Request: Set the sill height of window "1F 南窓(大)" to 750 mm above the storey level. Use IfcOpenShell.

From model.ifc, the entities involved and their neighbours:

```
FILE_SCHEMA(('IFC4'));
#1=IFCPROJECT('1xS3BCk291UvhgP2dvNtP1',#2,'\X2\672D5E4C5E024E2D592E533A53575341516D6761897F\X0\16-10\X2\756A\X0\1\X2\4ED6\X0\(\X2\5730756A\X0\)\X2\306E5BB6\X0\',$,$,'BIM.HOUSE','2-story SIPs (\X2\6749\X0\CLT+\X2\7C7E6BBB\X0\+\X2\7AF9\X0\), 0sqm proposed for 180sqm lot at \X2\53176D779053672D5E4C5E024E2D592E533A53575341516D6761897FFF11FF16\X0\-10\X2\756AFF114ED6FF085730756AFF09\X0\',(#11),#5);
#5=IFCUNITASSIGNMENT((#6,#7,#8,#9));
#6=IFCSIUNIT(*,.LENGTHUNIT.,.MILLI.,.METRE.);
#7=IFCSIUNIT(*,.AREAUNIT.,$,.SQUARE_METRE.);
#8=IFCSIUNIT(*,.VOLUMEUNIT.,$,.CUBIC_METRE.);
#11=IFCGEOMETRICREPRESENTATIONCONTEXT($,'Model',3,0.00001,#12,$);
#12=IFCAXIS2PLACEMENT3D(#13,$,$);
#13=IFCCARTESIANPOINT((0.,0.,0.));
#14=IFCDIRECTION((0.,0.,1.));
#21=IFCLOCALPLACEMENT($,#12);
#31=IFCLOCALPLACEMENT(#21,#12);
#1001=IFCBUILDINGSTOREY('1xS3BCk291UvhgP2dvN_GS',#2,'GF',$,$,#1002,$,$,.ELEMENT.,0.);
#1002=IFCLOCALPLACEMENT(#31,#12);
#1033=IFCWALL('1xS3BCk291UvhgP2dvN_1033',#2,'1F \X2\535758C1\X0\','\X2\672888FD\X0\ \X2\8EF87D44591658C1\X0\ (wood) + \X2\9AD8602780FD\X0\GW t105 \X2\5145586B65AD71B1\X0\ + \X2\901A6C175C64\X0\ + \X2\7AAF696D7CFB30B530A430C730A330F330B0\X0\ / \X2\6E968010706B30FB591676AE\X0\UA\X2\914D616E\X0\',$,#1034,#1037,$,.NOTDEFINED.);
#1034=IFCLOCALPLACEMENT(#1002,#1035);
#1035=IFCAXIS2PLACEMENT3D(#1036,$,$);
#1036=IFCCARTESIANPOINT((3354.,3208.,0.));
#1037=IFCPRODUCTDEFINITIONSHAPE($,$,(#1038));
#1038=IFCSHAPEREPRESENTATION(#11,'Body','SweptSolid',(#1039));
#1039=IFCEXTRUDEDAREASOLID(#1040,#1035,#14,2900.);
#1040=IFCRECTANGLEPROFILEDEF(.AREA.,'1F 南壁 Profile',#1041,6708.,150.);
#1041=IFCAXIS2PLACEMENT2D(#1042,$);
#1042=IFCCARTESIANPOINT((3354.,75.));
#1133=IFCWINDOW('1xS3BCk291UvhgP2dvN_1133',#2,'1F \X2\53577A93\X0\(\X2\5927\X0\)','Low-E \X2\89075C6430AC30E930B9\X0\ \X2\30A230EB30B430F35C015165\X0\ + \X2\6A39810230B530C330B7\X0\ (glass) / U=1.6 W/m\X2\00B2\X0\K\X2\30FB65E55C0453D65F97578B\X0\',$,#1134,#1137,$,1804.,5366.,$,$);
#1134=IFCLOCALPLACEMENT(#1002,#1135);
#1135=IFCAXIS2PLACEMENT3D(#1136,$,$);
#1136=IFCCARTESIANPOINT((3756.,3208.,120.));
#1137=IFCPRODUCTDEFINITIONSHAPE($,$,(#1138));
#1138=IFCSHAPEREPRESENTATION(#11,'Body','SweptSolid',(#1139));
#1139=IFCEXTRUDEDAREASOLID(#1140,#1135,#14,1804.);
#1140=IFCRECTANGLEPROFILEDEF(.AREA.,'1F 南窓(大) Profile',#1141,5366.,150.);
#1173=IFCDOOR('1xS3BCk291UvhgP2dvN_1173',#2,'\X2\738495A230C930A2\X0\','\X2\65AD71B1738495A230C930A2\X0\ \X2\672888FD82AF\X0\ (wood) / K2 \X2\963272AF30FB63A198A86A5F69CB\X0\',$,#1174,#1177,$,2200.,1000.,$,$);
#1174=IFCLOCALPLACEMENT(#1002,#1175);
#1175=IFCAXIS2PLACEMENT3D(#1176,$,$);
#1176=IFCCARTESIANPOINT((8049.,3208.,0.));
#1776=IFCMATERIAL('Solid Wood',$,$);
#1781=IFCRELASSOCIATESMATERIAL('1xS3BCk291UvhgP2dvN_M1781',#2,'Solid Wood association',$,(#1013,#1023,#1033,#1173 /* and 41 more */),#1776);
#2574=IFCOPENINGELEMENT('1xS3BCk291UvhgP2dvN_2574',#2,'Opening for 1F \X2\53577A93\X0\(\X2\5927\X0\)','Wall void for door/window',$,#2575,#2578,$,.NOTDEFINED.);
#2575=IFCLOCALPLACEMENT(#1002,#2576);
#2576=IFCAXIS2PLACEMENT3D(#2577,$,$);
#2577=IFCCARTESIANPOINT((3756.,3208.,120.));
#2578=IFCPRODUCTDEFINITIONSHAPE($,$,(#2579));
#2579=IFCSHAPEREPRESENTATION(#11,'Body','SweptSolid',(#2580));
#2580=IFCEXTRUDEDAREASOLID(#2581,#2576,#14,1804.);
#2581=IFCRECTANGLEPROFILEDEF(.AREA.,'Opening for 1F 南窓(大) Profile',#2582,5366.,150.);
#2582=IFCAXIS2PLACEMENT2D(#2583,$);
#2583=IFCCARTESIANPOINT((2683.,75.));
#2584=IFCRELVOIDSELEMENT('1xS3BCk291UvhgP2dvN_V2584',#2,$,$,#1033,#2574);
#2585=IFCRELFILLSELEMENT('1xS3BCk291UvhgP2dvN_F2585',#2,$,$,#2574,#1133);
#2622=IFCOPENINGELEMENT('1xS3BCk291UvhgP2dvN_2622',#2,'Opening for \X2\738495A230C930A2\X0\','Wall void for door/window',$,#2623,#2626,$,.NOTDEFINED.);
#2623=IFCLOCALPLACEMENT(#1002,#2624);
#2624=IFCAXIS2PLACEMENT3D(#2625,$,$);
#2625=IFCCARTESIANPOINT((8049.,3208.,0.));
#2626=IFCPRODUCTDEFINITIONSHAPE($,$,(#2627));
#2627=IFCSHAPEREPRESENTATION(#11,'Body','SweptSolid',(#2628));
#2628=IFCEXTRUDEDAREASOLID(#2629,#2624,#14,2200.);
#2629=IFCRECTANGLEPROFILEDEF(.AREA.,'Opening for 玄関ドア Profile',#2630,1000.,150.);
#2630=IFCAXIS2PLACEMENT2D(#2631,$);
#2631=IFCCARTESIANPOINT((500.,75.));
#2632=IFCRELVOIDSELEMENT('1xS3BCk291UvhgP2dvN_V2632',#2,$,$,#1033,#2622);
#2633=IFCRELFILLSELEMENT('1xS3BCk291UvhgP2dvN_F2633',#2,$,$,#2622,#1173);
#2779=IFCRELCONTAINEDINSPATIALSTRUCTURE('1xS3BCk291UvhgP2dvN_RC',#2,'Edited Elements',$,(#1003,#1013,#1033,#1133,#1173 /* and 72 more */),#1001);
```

```python
import numpy as np
import ifcopenshell
import ifcopenshell.api.geometry
import ifcopenshell.geom
import ifcopenshell.util.element
import ifcopenshell.util.placement
import ifcopenshell.util.shape
import ifcopenshell.util.unit

model = ifcopenshell.open("model.ifc")
unit_scale = ifcopenshell.util.unit.calculate_unit_scale(model)

window = model.by_id(1133)
opening = window.FillsVoids[0].RelatingOpeningElement
storey = ifcopenshell.util.element.get_container(window, ifc_class="IfcBuildingStorey")
level = ifcopenshell.util.placement.get_local_placement(storey.ObjectPlacement)[2, 3]

# The opening's origin need not be at the sill, so measure its lowest point.
shape = ifcopenshell.geom.create_shape(ifcopenshell.geom.settings(), opening)
bottom = ifcopenshell.util.shape.get_shape_bottom_elevation(shape, shape.geometry) / unit_scale
dz = level + 750.0 - bottom

shift = np.array([0.0, 0.0, dz])
# The window is not placed relative to its opening, so move both.
for product in (opening, window):
    matrix = ifcopenshell.util.placement.get_local_placement(product.ObjectPlacement)
    matrix[:3, 3] += shift
    ifcopenshell.api.geometry.edit_object_placement(model, product=product, matrix=matrix, is_si=False)

print(f"moved by {dz * unit_scale:+.3f} m")

model.write("model_edited.ifc")
```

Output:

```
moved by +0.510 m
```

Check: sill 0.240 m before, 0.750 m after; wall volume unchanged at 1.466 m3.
